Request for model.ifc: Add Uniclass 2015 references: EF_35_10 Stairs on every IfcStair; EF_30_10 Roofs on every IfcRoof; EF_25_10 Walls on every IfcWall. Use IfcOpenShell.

First a look at what the model holds.

```python
import ifcopenshell

model = ifcopenshell.open("model.ifc")
print(model.schema)
print("classifications:", [c.Name for c in model.by_type("IfcClassification")])
for ifc_class in ("IfcDoor", "IfcRoof", "IfcStair", "IfcWall", "IfcWindow"):
    print(ifc_class, len(model.by_type(ifc_class)))
```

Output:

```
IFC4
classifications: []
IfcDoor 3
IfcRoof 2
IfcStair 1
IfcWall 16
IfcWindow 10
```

```python
import ifcopenshell
import ifcopenshell.api.classification

model = ifcopenshell.open("model.ifc")

system = ifcopenshell.api.classification.add_classification(model, classification="Uniclass 2015")

codes = {
    "IfcStair": ("EF_35_10", "Stairs"),
    "IfcRoof": ("EF_30_10", "Roofs"),
    "IfcWall": ("EF_25_10", "Walls"),
}
for ifc_class, (code, name) in codes.items():
    products = model.by_type(ifc_class)
    ifcopenshell.api.classification.add_reference(
        model, products=products, classification=system, identification=code, name=name
    )
    print(code, len(products))

model.write("model_rev.ifc")
```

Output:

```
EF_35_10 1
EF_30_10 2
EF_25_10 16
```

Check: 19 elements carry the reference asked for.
